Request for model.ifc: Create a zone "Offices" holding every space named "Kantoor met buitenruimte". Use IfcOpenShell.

First a look at what the model holds.

```python
import ifcopenshell

model = ifcopenshell.open("model.ifc")
print(model.schema)
seen = {}
for space in model.by_type("IfcSpace"):
    seen[space.LongName] = seen.get(space.LongName, 0) + 1
for name, count in sorted(seen.items(), key=str):
    print(count, "x", name)
print("zones:", [z.Name for z in model.by_type("IfcZone")][:20])
```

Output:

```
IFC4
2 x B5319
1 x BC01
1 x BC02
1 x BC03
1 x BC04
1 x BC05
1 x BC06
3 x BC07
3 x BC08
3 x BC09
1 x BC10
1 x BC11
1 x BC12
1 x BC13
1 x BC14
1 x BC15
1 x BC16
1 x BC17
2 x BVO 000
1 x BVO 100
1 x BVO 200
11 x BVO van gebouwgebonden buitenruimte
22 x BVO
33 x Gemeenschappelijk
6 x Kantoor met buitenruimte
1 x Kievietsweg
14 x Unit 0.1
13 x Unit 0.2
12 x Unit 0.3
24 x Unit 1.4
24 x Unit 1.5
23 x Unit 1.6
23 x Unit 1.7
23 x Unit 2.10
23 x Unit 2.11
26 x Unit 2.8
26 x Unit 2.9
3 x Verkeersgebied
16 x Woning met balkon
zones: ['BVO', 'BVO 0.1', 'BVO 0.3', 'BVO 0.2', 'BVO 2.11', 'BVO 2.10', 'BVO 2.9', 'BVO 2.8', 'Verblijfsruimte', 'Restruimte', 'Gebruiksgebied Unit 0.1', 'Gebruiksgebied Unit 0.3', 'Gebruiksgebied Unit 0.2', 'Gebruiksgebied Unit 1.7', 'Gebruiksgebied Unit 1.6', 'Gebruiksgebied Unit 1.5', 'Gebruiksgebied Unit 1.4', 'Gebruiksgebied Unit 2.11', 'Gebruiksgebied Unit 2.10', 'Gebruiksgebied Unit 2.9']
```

```python
import ifcopenshell
import ifcopenshell.api.group
import ifcopenshell.api.root

model = ifcopenshell.open("model.ifc")

names = {"Kantoor met buitenruimte"}
spaces = [s for s in model.by_type("IfcSpace") if s.LongName in names]

zone = ifcopenshell.api.root.create_entity(model, ifc_class="IfcZone", name="Offices")
ifcopenshell.api.group.assign_group(model, products=spaces, group=zone)
print(len(spaces), "spaces in", zone.Name)

model.write("model-out.ifc")
```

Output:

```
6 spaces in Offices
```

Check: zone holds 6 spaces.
